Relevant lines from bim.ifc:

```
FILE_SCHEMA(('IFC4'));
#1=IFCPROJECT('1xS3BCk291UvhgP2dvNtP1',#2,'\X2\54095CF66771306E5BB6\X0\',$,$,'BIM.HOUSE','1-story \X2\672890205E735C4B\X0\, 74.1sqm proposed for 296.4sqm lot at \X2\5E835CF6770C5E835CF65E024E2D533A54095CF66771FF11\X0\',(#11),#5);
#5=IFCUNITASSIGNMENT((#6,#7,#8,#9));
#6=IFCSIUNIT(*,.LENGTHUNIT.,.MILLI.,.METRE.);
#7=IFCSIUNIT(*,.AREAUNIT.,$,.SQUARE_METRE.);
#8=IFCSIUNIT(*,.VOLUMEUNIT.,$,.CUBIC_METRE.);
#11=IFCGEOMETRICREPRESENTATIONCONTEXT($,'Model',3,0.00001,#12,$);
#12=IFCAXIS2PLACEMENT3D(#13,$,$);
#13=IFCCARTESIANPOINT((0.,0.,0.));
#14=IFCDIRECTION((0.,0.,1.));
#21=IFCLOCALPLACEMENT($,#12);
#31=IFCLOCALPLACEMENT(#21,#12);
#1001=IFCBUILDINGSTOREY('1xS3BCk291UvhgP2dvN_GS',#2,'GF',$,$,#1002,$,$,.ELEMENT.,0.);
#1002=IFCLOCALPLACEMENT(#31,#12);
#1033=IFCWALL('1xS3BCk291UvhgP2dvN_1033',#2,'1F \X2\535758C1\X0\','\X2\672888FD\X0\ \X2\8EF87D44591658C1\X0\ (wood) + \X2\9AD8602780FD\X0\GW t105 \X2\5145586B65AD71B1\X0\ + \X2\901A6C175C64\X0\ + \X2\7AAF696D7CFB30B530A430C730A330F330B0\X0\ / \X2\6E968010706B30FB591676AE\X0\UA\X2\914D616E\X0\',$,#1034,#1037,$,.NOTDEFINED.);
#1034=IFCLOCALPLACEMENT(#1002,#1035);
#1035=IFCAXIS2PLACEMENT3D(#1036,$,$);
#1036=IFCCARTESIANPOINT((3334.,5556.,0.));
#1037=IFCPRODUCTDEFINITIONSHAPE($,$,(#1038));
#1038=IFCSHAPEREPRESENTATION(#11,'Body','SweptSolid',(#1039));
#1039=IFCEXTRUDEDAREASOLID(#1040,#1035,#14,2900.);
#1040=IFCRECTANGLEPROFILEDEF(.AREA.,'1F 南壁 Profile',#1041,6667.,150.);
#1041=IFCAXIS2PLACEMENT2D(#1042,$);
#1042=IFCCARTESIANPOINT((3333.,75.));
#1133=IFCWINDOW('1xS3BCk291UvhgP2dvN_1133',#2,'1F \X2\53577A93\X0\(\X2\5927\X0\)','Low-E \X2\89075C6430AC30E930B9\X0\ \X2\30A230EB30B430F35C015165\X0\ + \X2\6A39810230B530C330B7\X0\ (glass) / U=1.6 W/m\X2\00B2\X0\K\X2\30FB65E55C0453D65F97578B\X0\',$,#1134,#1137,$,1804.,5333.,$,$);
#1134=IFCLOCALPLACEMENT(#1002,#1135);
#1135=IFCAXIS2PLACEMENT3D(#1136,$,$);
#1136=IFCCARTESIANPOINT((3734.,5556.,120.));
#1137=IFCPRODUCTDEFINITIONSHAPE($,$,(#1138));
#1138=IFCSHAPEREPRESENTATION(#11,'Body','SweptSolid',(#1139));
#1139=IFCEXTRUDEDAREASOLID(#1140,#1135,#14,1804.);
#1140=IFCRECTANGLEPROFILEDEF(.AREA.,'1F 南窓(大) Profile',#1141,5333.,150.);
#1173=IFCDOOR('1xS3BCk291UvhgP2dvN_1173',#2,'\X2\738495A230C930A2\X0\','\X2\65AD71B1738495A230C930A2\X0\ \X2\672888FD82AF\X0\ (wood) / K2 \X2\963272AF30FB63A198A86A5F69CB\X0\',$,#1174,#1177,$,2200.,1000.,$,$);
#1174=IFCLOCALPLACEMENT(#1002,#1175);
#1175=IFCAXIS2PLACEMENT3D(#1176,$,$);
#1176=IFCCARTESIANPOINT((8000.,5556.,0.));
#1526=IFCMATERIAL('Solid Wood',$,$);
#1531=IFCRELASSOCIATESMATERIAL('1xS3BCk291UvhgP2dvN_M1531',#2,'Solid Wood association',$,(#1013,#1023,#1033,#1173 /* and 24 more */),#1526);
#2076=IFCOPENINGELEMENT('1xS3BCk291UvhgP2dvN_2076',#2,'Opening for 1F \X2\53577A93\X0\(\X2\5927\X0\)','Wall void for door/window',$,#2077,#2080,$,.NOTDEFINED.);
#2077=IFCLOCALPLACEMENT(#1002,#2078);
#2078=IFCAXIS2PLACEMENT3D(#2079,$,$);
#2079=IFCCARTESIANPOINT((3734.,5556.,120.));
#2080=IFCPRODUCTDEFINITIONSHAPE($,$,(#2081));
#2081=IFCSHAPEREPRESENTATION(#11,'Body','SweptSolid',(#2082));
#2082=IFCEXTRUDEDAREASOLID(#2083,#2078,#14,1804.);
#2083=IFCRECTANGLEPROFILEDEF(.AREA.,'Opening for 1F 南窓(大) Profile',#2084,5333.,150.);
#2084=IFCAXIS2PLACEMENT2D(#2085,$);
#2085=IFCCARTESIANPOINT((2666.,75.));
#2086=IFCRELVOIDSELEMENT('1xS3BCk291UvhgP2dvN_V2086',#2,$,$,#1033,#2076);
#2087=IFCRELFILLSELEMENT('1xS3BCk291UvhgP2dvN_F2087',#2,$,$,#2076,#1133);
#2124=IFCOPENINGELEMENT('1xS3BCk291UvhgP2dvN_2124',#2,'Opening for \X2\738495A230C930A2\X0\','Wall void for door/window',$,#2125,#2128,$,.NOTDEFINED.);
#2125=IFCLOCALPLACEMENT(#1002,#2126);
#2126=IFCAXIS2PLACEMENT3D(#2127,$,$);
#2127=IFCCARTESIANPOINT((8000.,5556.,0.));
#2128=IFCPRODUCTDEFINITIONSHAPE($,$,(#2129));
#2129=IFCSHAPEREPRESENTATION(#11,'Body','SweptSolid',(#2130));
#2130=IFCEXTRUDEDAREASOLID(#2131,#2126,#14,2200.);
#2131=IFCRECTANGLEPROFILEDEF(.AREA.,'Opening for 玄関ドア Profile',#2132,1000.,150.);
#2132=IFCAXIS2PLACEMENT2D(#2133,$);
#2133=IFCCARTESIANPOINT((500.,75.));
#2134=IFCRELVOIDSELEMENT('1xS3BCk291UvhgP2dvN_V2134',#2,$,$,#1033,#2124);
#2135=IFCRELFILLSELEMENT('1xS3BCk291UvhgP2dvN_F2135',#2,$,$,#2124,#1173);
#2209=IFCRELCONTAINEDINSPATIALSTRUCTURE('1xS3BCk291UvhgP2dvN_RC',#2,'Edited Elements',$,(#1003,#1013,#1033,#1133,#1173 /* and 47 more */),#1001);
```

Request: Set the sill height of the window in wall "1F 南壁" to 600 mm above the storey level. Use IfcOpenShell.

```python
import numpy as np
import ifcopenshell
import ifcopenshell.api.geometry
import ifcopenshell.geom
import ifcopenshell.util.element
import ifcopenshell.util.placement
import ifcopenshell.util.shape
import ifcopenshell.util.unit

model = ifcopenshell.open("bim.ifc")
unit_scale = ifcopenshell.util.unit.calculate_unit_scale(model)

window = model.by_guid("1xS3BCk291UvhgP2dvN_1133")
opening = window.FillsVoids[0].RelatingOpeningElement
storey = ifcopenshell.util.element.get_container(window, ifc_class="IfcBuildingStorey")
level = ifcopenshell.util.placement.get_local_placement(storey.ObjectPlacement)[2, 3]

# The opening's origin need not be at the sill, so measure its lowest point.
shape = ifcopenshell.geom.create_shape(ifcopenshell.geom.settings(), opening)
bottom = ifcopenshell.util.shape.get_shape_bottom_elevation(shape, shape.geometry) / unit_scale
dz = level + 0.6 / unit_scale - bottom

shift = np.array([0.0, 0.0, dz])
# The window is not placed relative to its opening, so move both.
for product in (opening, window):
    matrix = ifcopenshell.util.placement.get_local_placement(product.ObjectPlacement)
    matrix[:3, 3] += shift
    ifcopenshell.api.geometry.edit_object_placement(model, product=product, matrix=matrix, is_si=False)

print(f"moved by {dz * unit_scale:+.3f} m")

model.write("bim_rev.ifc")
```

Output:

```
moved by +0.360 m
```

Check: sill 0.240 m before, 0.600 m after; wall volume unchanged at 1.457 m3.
